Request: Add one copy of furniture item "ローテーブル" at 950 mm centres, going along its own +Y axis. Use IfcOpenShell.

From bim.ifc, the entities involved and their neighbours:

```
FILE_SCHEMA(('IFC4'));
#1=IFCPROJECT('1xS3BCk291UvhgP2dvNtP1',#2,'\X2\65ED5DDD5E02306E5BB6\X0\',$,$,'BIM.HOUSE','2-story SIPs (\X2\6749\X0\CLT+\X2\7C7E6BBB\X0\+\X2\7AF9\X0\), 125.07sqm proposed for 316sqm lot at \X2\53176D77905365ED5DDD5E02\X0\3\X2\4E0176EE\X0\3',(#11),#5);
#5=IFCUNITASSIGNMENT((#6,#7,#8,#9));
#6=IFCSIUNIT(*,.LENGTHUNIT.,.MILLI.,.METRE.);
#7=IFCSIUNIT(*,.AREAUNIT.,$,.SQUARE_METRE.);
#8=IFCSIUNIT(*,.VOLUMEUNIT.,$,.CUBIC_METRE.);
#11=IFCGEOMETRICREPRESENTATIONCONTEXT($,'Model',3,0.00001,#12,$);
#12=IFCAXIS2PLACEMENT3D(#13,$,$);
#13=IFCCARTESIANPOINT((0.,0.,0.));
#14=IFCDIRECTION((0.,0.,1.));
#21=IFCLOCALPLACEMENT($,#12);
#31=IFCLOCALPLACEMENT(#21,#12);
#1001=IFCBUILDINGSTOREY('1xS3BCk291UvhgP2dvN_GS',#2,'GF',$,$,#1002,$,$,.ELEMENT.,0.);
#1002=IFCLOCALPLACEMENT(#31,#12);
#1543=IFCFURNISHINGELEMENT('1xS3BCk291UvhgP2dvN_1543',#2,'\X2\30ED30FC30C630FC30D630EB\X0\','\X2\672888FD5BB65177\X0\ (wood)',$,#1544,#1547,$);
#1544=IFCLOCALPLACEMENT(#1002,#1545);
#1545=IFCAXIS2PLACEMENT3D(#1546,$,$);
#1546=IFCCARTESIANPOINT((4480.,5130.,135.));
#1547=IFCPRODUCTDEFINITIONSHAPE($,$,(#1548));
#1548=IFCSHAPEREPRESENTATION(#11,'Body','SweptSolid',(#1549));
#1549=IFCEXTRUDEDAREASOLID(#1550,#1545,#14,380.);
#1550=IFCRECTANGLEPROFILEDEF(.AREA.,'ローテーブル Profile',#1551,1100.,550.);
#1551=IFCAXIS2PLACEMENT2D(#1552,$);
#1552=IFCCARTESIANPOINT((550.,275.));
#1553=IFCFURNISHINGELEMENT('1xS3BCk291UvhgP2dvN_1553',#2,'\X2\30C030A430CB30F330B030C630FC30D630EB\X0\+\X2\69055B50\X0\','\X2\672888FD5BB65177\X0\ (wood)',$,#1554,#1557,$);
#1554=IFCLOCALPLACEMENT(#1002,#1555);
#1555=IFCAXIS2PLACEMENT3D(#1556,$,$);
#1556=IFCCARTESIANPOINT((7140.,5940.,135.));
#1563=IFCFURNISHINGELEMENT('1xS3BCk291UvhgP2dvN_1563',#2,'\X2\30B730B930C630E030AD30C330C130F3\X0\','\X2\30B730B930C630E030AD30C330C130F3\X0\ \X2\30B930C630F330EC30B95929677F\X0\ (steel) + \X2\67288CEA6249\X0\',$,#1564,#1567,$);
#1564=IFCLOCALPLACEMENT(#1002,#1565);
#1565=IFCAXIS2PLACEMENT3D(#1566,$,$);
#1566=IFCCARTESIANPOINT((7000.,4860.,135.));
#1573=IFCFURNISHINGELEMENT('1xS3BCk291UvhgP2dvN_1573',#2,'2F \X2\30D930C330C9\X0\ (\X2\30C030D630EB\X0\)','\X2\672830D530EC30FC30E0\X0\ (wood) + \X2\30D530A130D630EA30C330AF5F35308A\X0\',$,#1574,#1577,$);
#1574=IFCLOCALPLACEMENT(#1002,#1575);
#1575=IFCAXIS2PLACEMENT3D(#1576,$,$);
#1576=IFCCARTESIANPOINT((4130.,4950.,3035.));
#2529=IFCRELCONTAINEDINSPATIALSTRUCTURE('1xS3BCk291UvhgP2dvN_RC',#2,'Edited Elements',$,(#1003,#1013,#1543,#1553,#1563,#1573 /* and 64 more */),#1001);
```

```python
import ifcopenshell
import ifcopenshell.api.geometry
import ifcopenshell.api.root
import ifcopenshell.util.element
import ifcopenshell.util.placement

model = ifcopenshell.open("bim.ifc")


def reuse_history(source, copy):
    """copy_class also copies each property set's owner history, people and application; keep the originals."""
    for rel in copy.IsDefinedBy:
        if rel.is_a("IfcRelDefinesByProperties") and (history := rel.RelatingPropertyDefinition.OwnerHistory):
            rel.RelatingPropertyDefinition.OwnerHistory = source.OwnerHistory
            ifcopenshell.util.element.remove_deep2(model, history)


source = model.by_guid("1xS3BCk291UvhgP2dvN_1543")
base = ifcopenshell.util.placement.get_local_placement(source.ObjectPlacement)
step = base[:3, 1] * 950.0

for i in range(1, 2):
    copy = ifcopenshell.api.root.copy_class(model, product=source)
    copy.Representation = ifcopenshell.util.element.copy_deep(
        model, source.Representation, exclude=["IfcGeometricRepresentationContext", "IfcRepresentationMap"]
    )
    reuse_history(source, copy)
    matrix = base.copy()
    matrix[:3, 3] += i * step
    print("added at", matrix[:3, 3].round(3) + 0.0)
    ifcopenshell.api.geometry.edit_object_placement(model, product=copy, matrix=matrix, is_si=False)

model.write("bim_updated.ifc")
```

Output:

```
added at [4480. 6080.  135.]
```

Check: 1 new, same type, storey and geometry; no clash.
